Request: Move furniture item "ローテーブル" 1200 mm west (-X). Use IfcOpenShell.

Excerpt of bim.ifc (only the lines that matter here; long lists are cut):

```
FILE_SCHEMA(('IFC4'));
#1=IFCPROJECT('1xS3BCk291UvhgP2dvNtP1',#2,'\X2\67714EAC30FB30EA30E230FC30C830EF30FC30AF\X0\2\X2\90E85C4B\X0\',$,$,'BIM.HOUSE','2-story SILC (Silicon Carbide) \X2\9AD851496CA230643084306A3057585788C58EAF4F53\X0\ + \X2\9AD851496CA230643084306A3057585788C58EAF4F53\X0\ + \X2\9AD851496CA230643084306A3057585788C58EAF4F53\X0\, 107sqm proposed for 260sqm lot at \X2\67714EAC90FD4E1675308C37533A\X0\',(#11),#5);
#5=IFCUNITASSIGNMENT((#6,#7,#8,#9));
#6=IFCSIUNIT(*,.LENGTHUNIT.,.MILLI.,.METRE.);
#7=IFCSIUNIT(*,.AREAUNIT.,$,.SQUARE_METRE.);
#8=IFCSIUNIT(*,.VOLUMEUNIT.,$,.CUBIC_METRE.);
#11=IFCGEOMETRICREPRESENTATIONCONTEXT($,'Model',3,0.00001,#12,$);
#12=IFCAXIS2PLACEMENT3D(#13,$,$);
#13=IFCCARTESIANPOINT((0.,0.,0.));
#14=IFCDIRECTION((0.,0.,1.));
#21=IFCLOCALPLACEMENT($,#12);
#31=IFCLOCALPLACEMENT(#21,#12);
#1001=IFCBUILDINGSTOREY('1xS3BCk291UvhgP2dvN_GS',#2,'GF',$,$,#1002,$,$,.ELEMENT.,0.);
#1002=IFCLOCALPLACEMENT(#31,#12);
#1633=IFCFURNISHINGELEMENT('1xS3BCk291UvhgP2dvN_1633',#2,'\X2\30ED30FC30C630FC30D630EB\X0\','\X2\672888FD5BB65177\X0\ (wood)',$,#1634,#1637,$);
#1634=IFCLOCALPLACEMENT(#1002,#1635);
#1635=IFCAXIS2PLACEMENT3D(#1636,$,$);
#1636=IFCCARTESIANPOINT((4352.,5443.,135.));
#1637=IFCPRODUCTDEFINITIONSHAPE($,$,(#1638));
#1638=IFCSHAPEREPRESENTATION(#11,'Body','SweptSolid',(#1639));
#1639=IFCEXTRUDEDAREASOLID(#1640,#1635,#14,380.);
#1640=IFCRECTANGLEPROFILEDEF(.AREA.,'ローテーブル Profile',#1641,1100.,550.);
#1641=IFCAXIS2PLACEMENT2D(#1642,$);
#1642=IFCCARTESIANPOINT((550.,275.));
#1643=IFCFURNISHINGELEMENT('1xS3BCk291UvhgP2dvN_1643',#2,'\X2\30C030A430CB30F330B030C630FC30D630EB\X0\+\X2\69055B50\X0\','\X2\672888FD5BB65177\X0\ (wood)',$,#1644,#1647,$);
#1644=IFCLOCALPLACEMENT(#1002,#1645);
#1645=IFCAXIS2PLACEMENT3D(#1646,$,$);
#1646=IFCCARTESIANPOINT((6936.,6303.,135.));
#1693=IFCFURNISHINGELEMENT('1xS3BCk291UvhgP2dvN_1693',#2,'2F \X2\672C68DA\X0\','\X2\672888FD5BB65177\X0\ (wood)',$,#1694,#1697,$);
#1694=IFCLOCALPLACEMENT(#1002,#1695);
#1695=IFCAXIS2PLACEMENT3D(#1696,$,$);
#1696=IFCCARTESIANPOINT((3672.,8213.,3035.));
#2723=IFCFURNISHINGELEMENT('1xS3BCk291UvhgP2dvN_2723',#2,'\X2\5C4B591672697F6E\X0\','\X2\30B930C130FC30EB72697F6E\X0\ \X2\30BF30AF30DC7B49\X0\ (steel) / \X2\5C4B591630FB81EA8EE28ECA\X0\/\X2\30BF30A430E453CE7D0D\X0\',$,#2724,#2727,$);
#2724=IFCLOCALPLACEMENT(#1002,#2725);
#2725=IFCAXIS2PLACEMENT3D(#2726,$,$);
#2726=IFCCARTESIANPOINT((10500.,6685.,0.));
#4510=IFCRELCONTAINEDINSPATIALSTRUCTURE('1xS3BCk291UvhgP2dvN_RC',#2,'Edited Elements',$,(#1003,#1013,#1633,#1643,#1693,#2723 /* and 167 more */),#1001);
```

```python
import ifcopenshell
import ifcopenshell.api.geometry
import ifcopenshell.util.placement

model = ifcopenshell.open("bim.ifc")

item = model.by_guid("1xS3BCk291UvhgP2dvN_1633")
matrix = ifcopenshell.util.placement.get_local_placement(item.ObjectPlacement)
matrix[0, 3] -= 1200.0
ifcopenshell.api.geometry.edit_object_placement(model, product=item, matrix=matrix, is_si=False)

print(ifcopenshell.util.placement.get_local_placement(item.ObjectPlacement).round(3) + 0.0)

model.write("bim_rev.ifc")
```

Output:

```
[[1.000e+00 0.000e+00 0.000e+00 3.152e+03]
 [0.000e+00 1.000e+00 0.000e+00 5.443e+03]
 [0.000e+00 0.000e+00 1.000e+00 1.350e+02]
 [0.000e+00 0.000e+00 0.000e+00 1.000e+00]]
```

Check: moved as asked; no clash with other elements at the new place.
